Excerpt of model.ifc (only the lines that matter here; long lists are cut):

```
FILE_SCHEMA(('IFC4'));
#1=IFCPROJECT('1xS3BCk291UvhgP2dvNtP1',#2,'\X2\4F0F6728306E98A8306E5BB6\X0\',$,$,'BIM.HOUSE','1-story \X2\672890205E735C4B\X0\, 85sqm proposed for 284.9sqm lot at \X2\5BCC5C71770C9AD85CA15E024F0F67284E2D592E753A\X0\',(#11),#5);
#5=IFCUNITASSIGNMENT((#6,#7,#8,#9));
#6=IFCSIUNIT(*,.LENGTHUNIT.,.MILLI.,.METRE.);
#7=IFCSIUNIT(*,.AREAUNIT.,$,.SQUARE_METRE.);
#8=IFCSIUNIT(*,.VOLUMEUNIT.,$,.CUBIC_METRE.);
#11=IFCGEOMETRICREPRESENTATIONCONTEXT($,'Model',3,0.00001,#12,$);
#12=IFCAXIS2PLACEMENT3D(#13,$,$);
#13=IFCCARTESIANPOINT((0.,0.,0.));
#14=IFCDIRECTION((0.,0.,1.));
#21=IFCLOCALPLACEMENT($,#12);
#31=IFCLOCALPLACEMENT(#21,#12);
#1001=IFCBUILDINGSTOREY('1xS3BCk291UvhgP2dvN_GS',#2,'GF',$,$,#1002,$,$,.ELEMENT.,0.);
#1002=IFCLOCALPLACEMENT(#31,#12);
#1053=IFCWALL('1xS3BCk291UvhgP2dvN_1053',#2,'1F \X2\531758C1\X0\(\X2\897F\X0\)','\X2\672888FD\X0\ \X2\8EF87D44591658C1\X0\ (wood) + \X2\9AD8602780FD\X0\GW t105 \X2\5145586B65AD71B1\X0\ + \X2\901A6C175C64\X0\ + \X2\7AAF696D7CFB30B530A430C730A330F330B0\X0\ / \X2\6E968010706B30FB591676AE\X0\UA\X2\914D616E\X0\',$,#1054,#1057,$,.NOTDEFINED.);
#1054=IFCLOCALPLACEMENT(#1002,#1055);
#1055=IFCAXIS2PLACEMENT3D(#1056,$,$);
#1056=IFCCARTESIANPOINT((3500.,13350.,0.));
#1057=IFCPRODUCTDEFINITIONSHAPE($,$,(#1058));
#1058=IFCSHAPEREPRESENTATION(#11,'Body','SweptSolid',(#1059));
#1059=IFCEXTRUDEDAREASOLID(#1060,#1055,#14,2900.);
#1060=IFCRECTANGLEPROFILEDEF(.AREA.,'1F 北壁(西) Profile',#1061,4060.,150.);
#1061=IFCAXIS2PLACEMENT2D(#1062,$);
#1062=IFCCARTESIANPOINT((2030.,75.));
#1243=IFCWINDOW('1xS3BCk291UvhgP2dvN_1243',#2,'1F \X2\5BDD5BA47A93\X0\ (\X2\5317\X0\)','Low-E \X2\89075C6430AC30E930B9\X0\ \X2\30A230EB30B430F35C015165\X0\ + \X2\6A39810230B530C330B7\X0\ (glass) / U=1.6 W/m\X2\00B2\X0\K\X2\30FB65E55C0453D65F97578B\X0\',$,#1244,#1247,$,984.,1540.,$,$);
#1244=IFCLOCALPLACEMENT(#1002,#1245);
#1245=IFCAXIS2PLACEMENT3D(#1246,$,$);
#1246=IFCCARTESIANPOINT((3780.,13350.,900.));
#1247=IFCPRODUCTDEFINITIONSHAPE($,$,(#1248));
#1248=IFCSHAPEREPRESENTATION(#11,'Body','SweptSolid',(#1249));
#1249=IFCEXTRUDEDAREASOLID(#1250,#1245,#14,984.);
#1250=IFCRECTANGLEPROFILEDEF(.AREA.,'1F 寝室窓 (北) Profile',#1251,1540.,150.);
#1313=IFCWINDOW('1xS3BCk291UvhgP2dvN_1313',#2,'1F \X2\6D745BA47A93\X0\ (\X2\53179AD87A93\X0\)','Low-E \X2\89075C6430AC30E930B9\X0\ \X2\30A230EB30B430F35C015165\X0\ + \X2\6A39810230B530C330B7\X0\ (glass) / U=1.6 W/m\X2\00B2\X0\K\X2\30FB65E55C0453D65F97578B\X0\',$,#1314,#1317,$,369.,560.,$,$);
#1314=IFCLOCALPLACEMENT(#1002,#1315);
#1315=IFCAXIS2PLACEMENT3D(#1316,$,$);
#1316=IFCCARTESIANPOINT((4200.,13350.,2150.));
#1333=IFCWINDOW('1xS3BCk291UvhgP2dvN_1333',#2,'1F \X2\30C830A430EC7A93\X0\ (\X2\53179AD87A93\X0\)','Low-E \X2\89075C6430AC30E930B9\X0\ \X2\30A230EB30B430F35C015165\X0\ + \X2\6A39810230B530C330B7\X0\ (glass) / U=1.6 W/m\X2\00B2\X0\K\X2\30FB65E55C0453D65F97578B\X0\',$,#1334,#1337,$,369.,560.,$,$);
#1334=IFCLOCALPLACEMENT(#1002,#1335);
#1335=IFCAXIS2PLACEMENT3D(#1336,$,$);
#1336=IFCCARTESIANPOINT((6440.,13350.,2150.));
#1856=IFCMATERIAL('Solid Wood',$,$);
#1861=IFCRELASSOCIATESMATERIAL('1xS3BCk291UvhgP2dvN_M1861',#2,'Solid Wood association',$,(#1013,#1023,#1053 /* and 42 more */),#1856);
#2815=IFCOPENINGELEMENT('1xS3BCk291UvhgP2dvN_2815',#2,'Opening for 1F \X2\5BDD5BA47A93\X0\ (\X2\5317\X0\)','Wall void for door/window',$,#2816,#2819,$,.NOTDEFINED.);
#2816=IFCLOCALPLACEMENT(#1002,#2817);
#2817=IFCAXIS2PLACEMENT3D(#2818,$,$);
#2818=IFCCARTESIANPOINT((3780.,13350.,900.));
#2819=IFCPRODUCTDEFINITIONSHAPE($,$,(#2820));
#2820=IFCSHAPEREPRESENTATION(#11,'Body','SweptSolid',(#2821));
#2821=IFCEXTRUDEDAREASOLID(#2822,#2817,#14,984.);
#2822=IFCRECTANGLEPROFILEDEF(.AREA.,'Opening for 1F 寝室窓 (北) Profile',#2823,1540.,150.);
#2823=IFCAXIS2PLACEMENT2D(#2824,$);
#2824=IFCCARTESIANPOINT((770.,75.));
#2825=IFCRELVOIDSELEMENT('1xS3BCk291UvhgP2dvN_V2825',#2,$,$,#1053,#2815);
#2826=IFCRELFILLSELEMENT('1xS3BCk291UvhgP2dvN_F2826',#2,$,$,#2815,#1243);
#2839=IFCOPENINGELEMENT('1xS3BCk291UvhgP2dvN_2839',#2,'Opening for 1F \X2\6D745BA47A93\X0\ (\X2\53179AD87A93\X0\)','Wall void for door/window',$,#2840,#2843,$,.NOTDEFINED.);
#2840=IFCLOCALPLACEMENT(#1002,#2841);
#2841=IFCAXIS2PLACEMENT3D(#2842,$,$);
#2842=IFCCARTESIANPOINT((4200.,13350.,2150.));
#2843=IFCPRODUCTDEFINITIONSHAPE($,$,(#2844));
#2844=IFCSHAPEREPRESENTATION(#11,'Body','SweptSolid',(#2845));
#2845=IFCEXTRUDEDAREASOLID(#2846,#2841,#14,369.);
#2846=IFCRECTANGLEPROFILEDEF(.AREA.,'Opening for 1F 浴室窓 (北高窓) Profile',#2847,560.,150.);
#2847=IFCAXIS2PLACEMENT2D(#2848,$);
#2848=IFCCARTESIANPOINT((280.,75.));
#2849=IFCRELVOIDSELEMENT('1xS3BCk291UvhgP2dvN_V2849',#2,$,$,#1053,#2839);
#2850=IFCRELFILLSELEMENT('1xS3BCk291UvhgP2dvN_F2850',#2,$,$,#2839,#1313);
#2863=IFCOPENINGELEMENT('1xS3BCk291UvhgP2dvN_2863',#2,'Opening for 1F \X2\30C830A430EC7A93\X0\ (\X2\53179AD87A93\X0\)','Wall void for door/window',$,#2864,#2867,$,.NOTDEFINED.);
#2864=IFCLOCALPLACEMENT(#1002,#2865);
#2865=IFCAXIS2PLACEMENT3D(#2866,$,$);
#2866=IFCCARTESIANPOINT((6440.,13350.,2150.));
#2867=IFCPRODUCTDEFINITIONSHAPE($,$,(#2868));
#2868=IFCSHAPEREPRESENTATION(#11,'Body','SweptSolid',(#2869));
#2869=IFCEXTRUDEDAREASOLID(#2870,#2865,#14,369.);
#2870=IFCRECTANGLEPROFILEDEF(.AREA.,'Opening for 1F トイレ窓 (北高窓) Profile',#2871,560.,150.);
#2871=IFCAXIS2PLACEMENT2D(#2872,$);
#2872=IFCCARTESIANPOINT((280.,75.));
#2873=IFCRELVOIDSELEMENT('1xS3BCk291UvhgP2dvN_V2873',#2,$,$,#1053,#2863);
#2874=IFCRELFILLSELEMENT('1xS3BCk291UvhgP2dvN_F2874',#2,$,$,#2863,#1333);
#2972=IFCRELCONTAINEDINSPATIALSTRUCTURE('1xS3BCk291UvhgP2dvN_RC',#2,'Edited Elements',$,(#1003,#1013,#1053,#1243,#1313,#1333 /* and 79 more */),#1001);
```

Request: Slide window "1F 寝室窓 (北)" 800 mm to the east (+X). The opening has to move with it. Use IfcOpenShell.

```python
import ifcopenshell
import ifcopenshell.api.geometry
import ifcopenshell.util.placement
import ifcopenshell.util.unit

model = ifcopenshell.open("model.ifc")
unit_scale = ifcopenshell.util.unit.calculate_unit_scale(model)

window = model.by_guid("1xS3BCk291UvhgP2dvN_1243")
opening = window.FillsVoids[0].RelatingOpeningElement
wall = opening.VoidsElements[0].RelatingBuildingElement

wall_matrix = ifcopenshell.util.placement.get_local_placement(wall.ObjectPlacement)
shift = wall_matrix[:3, 0] * 0.8 / unit_scale
before = ifcopenshell.util.placement.get_local_placement(window.ObjectPlacement)[:3, 3].copy()

# The window is not placed relative to its opening, so move both.
for product in (opening, window):
    matrix = ifcopenshell.util.placement.get_local_placement(product.ObjectPlacement)
    matrix[:3, 3] += shift
    ifcopenshell.api.geometry.edit_object_placement(model, product=product, matrix=matrix, is_si=False)

after = ifcopenshell.util.placement.get_local_placement(window.ObjectPlacement)[:3, 3]
print("window moved by", (after - before).round(3) + 0.0)

model.write("model_edited.ifc")
```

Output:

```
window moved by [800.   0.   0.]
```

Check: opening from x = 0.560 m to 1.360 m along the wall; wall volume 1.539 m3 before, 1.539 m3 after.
